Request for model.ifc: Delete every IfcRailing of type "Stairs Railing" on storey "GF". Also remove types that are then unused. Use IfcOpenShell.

First a look at what the model holds.

```python
import ifcopenshell
import ifcopenshell.util.element

model = ifcopenshell.open("model.ifc")
print(model.schema)
storey = next(s for s in model.by_type("IfcBuildingStorey") if s.Name == "GF")
railings = [e for e in ifcopenshell.util.element.get_decomposition(storey) if e.is_a("IfcRailing")]
seen = {}
for e in railings:
    element_type = ifcopenshell.util.element.get_type(e)
    name = element_type.Name if element_type not in (None, e) else None
    seen[name] = seen.get(name, 0) + 1
for name, count in sorted(seen.items(), key=str):
    print(count, "x", name)
```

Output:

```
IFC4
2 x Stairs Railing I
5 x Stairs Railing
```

```python
import ifcopenshell
import ifcopenshell.api.root
import ifcopenshell.util.element

model = ifcopenshell.open("model.ifc")

storey = next(s for s in model.by_type("IfcBuildingStorey") if s.Name == "GF")
railings = [e for e in ifcopenshell.util.element.get_decomposition(storey) if e.is_a("IfcRailing")]
targets = [e for e in railings if (t := ifcopenshell.util.element.get_type(e)) not in (None, e) and t.Name == "Stairs Railing"]
types = {ifcopenshell.util.element.get_type(e) for e in targets} - {None, *targets}

for e in targets:
    ifcopenshell.api.root.remove_product(model, product=e)
print(len(targets), "removed")

unused = [t for t in types if not ifcopenshell.util.element.get_types(t)]
for t in unused:
    ifcopenshell.api.root.remove_product(model, product=t)
print(len(unused), "unused types removed")

model.write("model-out.ifc")
```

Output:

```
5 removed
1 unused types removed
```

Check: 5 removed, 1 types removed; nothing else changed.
